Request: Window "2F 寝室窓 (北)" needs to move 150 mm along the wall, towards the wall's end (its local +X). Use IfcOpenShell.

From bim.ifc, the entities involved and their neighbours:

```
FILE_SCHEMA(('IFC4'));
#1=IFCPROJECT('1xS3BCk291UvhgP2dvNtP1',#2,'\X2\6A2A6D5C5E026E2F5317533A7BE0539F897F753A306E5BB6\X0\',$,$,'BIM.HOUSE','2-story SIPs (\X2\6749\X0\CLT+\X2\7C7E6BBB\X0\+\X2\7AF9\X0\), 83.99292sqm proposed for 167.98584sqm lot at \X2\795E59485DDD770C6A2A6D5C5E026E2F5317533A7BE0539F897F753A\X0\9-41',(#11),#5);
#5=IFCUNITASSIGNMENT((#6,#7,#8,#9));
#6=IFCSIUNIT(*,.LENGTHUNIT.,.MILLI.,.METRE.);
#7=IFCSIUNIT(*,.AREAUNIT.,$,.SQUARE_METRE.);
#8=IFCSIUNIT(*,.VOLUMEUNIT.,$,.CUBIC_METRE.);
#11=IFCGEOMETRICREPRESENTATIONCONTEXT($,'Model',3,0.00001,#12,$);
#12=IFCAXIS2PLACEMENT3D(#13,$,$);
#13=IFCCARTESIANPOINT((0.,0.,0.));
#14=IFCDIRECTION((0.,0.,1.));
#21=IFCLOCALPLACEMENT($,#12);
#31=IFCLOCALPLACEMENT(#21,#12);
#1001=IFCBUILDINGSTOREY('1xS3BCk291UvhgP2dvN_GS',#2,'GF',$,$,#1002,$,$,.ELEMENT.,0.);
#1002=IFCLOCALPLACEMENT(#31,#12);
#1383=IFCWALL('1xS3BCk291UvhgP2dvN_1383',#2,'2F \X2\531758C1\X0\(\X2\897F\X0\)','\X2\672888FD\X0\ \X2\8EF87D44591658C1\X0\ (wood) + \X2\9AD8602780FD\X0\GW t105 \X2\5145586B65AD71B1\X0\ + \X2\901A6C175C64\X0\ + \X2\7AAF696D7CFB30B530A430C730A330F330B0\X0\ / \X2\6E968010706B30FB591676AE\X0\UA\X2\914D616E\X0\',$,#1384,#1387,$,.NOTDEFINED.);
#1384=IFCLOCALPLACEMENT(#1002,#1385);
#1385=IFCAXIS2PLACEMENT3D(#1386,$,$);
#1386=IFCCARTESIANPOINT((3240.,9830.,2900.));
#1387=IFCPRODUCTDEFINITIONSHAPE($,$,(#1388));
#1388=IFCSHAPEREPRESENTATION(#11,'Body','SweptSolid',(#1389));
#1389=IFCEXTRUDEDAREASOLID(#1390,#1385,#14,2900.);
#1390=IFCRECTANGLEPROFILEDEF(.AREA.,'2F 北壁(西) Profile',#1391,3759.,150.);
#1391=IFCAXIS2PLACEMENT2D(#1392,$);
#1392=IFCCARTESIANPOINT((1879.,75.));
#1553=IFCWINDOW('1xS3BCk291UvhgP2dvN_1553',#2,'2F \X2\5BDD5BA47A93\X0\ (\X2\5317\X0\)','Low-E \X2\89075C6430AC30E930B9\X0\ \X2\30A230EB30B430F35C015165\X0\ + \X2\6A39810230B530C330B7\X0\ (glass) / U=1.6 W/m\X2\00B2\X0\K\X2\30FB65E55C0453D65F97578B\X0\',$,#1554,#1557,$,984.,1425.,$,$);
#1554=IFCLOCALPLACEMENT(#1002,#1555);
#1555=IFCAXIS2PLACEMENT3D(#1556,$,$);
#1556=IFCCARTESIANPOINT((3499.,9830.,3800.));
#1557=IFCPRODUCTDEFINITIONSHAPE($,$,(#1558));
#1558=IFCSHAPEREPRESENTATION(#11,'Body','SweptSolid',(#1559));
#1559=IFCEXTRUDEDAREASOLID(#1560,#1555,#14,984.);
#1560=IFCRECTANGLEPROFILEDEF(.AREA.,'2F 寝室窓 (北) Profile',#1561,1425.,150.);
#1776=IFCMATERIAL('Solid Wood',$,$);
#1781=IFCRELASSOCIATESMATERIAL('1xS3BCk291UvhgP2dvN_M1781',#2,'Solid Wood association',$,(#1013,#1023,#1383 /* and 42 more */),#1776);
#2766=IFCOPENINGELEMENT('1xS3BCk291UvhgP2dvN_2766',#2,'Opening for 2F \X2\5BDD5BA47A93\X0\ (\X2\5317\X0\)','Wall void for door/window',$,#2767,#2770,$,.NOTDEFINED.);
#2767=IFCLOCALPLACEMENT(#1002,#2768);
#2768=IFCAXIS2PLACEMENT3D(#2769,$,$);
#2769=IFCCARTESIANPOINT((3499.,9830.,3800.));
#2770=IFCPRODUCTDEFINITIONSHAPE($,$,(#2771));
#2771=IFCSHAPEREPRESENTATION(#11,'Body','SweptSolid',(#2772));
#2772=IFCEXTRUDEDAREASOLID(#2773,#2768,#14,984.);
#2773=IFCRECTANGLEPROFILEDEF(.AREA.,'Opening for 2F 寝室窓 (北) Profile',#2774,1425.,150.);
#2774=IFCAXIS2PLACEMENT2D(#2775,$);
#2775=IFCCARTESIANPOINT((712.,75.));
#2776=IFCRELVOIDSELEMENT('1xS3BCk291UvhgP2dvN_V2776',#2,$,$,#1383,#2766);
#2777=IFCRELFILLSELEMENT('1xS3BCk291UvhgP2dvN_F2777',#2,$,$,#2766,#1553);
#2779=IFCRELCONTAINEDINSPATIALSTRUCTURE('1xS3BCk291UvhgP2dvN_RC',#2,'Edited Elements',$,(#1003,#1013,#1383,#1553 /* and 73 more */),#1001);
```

```python
import ifcopenshell
import ifcopenshell.api.geometry
import ifcopenshell.util.placement

model = ifcopenshell.open("bim.ifc")

window = model.by_id(1553)
opening = window.FillsVoids[0].RelatingOpeningElement
wall = opening.VoidsElements[0].RelatingBuildingElement

wall_matrix = ifcopenshell.util.placement.get_local_placement(wall.ObjectPlacement)
shift = wall_matrix[:3, 0] * 150.0
before = ifcopenshell.util.placement.get_local_placement(window.ObjectPlacement)[:3, 3].copy()

# The window is not placed relative to its opening, so move both.
for product in (opening, window):
    matrix = ifcopenshell.util.placement.get_local_placement(product.ObjectPlacement)
    matrix[:3, 3] += shift
    ifcopenshell.api.geometry.edit_object_placement(model, product=product, matrix=matrix, is_si=False)

after = ifcopenshell.util.placement.get_local_placement(window.ObjectPlacement)[:3, 3]
print("window moved by", (after - before).round(3) + 0.0)

model.write("bim-out.ifc")
```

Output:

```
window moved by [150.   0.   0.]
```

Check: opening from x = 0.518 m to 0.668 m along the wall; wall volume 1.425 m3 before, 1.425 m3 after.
